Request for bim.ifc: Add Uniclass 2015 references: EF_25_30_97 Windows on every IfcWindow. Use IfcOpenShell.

First a look at what the model holds.

```python
import ifcopenshell

model = ifcopenshell.open("bim.ifc")
print(model.schema)
print("classifications:", [c.Name for c in model.by_type("IfcClassification")])
for ifc_class in ("IfcDoor", "IfcRoof", "IfcStair", "IfcWall", "IfcWindow"):
    print(ifc_class, len(model.by_type(ifc_class)))
```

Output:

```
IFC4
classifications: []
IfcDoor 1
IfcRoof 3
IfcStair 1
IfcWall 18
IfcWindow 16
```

```python
import ifcopenshell
import ifcopenshell.api.classification

model = ifcopenshell.open("bim.ifc")

system = ifcopenshell.api.classification.add_classification(model, classification="Uniclass 2015")

codes = {
    "IfcWindow": ("EF_25_30_97", "Windows"),
}
for ifc_class, (code, name) in codes.items():
    products = model.by_type(ifc_class)
    ifcopenshell.api.classification.add_reference(
        model, products=products, classification=system, identification=code, name=name
    )
    print(code, len(products))

model.write("bim_updated.ifc")
```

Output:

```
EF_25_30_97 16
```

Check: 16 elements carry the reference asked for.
